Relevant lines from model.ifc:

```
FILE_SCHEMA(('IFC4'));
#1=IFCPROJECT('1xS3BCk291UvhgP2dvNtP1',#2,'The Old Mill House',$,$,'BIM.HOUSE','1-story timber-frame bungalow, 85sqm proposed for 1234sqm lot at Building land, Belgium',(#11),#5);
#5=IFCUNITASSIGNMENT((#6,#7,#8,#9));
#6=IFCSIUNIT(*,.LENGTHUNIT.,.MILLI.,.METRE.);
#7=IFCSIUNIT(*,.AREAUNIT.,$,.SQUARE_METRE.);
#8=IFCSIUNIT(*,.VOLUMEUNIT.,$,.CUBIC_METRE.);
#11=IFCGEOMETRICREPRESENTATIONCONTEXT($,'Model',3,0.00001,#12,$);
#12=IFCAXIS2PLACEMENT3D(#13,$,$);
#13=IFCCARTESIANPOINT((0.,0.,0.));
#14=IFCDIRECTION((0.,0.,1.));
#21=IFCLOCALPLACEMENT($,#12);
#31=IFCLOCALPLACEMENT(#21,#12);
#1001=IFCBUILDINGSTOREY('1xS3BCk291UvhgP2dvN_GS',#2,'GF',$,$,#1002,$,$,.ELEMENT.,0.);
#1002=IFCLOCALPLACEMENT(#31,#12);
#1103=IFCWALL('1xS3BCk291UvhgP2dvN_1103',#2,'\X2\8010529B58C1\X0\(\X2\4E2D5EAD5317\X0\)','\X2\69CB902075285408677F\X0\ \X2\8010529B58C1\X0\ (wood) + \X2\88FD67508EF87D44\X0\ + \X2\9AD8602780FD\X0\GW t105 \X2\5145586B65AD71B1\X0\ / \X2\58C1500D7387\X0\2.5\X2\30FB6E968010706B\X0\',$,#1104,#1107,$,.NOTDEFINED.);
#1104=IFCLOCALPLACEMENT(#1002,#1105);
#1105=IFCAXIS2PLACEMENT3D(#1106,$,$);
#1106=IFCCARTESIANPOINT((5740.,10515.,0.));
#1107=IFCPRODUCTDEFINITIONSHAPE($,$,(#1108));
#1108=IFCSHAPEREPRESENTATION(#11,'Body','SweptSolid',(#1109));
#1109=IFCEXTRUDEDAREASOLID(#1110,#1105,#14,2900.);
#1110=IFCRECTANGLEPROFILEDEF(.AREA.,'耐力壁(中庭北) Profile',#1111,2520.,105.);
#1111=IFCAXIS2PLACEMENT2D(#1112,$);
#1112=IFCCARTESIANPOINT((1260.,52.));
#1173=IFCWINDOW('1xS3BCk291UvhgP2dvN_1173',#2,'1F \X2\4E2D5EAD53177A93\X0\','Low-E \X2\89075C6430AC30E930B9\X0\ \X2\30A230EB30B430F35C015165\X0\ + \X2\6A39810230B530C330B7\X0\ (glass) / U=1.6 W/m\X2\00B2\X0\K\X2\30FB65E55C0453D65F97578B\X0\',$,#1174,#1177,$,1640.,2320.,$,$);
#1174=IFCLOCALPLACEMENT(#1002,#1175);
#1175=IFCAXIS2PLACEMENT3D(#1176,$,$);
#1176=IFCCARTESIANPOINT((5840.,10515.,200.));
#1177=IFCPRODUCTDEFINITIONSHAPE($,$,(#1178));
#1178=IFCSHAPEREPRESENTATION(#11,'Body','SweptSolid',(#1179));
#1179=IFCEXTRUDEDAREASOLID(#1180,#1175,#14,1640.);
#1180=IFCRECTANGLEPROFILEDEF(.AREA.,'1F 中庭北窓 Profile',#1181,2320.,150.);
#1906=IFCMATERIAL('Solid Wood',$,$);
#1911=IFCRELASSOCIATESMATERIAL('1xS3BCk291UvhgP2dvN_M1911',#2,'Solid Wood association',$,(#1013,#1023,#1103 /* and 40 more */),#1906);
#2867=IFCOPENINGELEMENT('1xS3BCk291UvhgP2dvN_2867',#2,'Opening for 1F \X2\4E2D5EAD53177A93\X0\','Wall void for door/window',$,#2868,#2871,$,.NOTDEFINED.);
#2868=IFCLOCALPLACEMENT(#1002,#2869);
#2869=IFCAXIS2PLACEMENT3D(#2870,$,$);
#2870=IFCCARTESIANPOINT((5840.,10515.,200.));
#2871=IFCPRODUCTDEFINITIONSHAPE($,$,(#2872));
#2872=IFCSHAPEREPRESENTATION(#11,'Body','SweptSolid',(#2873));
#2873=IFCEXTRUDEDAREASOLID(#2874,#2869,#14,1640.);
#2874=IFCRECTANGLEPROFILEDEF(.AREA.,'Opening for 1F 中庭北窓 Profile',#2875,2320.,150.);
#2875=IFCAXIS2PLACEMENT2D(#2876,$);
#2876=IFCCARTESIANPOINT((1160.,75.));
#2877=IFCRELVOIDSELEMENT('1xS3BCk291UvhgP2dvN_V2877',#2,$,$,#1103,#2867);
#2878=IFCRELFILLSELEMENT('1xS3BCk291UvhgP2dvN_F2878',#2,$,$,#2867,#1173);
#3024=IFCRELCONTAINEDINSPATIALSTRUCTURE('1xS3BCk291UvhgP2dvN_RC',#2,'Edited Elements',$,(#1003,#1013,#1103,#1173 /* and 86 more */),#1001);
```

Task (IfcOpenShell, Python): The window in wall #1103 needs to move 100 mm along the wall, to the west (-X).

```python
import ifcopenshell
import ifcopenshell.api.geometry
import ifcopenshell.util.placement

model = ifcopenshell.open("model.ifc")

window = model.by_guid("1xS3BCk291UvhgP2dvN_1173")
opening = window.FillsVoids[0].RelatingOpeningElement
wall = opening.VoidsElements[0].RelatingBuildingElement

wall_matrix = ifcopenshell.util.placement.get_local_placement(wall.ObjectPlacement)
shift = wall_matrix[:3, 0] * -100.0
before = ifcopenshell.util.placement.get_local_placement(window.ObjectPlacement)[:3, 3].copy()

# The window is not placed relative to its opening, so move both.
for product in (opening, window):
    matrix = ifcopenshell.util.placement.get_local_placement(product.ObjectPlacement)
    matrix[:3, 3] += shift
    ifcopenshell.api.geometry.edit_object_placement(model, product=product, matrix=matrix, is_si=False)

after = ifcopenshell.util.placement.get_local_placement(window.ObjectPlacement)[:3, 3]
print("window moved by", (after - before).round(3) + 0.0)

model.write("model_edited.ifc")
```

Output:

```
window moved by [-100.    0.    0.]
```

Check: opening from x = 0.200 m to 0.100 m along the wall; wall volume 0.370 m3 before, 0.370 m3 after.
